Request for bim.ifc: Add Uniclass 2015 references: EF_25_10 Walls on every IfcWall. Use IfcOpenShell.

First a look at what the model holds.

```python
import ifcopenshell

model = ifcopenshell.open("bim.ifc")
print(model.schema)
print("classifications:", [c.Name for c in model.by_type("IfcClassification")])
for ifc_class in ("IfcDoor", "IfcRoof", "IfcStair", "IfcWall", "IfcWindow"):
    print(ifc_class, len(model.by_type(ifc_class)))
```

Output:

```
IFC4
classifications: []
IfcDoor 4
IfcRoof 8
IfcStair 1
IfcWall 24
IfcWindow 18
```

```python
import ifcopenshell
import ifcopenshell.api.classification

model = ifcopenshell.open("bim.ifc")

system = ifcopenshell.api.classification.add_classification(model, classification="Uniclass 2015")

codes = {
    "IfcWall": ("EF_25_10", "Walls"),
}
for ifc_class, (code, name) in codes.items():
    products = model.by_type(ifc_class)
    ifcopenshell.api.classification.add_reference(
        model, products=products, classification=system, identification=code, name=name
    )
    print(code, len(products))

model.write("bim-out.ifc")
```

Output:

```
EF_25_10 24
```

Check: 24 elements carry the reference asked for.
